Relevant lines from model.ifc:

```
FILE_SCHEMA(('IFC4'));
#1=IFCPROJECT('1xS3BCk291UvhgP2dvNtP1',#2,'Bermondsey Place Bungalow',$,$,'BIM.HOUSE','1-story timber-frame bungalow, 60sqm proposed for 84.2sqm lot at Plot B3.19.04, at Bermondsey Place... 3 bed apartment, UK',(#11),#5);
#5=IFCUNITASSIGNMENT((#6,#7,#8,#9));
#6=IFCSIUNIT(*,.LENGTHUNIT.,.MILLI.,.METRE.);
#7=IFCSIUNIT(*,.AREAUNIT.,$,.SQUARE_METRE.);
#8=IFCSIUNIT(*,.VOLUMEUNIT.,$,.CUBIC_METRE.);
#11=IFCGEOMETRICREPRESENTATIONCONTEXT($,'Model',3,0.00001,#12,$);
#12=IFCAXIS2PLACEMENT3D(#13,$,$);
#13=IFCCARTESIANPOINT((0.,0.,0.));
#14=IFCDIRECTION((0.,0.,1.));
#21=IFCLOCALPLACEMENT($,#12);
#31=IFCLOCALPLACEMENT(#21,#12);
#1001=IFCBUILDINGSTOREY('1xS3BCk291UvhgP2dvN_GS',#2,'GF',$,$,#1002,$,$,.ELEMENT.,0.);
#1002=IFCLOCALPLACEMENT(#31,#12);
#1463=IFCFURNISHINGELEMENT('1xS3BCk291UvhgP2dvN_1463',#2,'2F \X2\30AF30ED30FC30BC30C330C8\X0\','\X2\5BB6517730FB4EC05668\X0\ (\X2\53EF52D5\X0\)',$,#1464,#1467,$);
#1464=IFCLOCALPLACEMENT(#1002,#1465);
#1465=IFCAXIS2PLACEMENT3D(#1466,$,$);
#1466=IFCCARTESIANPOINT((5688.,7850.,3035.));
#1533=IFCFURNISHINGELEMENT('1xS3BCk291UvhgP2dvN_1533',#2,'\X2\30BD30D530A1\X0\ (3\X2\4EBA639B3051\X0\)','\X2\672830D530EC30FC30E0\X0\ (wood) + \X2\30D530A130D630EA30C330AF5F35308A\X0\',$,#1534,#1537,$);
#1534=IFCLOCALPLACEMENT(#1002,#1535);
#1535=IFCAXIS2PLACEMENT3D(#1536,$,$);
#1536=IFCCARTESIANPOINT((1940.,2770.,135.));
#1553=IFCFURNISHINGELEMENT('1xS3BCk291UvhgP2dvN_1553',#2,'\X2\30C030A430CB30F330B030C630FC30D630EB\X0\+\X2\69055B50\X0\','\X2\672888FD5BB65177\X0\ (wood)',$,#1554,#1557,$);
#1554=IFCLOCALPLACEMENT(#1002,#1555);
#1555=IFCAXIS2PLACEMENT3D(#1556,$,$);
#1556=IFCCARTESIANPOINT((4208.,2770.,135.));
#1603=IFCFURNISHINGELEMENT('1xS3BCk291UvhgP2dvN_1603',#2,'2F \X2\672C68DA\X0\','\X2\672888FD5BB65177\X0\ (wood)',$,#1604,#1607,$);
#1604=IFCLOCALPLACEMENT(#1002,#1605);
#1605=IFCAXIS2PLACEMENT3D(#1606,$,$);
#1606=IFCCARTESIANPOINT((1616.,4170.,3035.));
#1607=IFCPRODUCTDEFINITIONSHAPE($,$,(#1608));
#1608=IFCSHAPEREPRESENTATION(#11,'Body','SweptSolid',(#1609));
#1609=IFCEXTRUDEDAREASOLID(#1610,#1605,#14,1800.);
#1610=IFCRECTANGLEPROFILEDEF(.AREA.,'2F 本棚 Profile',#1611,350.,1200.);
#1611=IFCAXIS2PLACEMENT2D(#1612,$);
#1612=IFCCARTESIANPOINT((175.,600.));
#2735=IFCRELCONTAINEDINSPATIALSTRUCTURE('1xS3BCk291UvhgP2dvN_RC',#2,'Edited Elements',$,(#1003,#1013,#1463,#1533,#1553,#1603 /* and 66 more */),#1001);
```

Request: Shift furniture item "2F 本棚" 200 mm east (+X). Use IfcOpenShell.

```python
import ifcopenshell
import ifcopenshell.api.geometry
import ifcopenshell.util.placement
import ifcopenshell.util.unit

model = ifcopenshell.open("model.ifc")
unit_scale = ifcopenshell.util.unit.calculate_unit_scale(model)

item = model.by_id(1603)
matrix = ifcopenshell.util.placement.get_local_placement(item.ObjectPlacement)
matrix[0, 3] += 0.2 / unit_scale
ifcopenshell.api.geometry.edit_object_placement(model, product=item, matrix=matrix, is_si=False)

print(ifcopenshell.util.placement.get_local_placement(item.ObjectPlacement).round(3) + 0.0)

model.write("model_rev.ifc")
```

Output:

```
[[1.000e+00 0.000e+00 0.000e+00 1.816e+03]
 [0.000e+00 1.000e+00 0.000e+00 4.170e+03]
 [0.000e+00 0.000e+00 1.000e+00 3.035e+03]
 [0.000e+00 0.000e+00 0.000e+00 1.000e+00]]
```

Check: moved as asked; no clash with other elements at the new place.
